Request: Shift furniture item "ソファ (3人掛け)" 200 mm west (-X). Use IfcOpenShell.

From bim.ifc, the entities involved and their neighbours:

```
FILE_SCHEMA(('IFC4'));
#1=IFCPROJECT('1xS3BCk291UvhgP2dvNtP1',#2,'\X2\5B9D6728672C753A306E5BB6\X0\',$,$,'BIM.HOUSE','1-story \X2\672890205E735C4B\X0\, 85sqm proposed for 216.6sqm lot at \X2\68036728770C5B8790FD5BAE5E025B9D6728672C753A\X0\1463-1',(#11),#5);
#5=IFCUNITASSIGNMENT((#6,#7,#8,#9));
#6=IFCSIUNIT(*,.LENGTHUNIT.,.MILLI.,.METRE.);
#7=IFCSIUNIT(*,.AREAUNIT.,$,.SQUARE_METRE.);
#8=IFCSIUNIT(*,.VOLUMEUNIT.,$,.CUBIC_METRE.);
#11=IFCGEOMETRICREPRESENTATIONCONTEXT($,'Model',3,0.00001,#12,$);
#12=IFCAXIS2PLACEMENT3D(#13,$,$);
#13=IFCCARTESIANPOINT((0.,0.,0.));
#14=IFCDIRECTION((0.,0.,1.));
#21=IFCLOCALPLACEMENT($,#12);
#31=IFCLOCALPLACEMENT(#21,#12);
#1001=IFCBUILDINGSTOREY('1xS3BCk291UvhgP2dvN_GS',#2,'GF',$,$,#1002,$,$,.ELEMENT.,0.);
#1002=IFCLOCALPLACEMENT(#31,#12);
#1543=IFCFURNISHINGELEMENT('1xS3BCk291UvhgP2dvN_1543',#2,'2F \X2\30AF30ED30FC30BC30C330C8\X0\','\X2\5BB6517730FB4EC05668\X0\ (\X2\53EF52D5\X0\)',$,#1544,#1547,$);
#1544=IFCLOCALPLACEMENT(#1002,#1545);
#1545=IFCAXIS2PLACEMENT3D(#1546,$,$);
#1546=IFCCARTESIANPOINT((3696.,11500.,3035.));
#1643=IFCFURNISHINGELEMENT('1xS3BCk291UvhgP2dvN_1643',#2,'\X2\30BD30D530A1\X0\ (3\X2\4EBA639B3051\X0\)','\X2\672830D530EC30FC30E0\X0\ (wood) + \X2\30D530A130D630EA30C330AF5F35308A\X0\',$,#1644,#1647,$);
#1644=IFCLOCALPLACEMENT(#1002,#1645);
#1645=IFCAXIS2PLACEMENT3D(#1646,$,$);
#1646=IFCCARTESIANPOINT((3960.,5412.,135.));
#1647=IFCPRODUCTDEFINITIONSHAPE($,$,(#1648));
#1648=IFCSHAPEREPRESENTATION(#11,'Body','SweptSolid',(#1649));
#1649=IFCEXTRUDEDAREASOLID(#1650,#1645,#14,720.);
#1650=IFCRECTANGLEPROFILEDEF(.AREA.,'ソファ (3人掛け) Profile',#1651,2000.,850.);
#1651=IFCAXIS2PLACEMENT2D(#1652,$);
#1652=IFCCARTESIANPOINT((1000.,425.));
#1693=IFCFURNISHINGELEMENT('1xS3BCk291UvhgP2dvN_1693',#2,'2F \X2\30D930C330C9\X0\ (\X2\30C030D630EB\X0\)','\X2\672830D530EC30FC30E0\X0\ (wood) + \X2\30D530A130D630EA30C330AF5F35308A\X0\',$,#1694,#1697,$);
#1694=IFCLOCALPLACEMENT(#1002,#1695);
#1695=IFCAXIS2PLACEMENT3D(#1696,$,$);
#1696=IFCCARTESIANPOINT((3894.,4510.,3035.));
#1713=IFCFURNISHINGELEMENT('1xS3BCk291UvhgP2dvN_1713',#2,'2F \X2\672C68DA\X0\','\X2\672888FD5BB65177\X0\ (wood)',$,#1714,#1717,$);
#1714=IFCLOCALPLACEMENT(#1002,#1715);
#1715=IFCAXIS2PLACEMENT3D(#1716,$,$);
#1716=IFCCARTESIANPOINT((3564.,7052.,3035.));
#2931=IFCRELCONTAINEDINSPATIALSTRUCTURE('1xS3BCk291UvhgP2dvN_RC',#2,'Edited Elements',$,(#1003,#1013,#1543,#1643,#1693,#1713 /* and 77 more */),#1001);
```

```python
import ifcopenshell
import ifcopenshell.api.geometry
import ifcopenshell.util.placement

model = ifcopenshell.open("bim.ifc")

item = model.by_id(1643)
matrix = ifcopenshell.util.placement.get_local_placement(item.ObjectPlacement)
matrix[0, 3] -= 200.0
ifcopenshell.api.geometry.edit_object_placement(model, product=item, matrix=matrix, is_si=False)

print(ifcopenshell.util.placement.get_local_placement(item.ObjectPlacement).round(3) + 0.0)

model.write("bim_v2.ifc")
```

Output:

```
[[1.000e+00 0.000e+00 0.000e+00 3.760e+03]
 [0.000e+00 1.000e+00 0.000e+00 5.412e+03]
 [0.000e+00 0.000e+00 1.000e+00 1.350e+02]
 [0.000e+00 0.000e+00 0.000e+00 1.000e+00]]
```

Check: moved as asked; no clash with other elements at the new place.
